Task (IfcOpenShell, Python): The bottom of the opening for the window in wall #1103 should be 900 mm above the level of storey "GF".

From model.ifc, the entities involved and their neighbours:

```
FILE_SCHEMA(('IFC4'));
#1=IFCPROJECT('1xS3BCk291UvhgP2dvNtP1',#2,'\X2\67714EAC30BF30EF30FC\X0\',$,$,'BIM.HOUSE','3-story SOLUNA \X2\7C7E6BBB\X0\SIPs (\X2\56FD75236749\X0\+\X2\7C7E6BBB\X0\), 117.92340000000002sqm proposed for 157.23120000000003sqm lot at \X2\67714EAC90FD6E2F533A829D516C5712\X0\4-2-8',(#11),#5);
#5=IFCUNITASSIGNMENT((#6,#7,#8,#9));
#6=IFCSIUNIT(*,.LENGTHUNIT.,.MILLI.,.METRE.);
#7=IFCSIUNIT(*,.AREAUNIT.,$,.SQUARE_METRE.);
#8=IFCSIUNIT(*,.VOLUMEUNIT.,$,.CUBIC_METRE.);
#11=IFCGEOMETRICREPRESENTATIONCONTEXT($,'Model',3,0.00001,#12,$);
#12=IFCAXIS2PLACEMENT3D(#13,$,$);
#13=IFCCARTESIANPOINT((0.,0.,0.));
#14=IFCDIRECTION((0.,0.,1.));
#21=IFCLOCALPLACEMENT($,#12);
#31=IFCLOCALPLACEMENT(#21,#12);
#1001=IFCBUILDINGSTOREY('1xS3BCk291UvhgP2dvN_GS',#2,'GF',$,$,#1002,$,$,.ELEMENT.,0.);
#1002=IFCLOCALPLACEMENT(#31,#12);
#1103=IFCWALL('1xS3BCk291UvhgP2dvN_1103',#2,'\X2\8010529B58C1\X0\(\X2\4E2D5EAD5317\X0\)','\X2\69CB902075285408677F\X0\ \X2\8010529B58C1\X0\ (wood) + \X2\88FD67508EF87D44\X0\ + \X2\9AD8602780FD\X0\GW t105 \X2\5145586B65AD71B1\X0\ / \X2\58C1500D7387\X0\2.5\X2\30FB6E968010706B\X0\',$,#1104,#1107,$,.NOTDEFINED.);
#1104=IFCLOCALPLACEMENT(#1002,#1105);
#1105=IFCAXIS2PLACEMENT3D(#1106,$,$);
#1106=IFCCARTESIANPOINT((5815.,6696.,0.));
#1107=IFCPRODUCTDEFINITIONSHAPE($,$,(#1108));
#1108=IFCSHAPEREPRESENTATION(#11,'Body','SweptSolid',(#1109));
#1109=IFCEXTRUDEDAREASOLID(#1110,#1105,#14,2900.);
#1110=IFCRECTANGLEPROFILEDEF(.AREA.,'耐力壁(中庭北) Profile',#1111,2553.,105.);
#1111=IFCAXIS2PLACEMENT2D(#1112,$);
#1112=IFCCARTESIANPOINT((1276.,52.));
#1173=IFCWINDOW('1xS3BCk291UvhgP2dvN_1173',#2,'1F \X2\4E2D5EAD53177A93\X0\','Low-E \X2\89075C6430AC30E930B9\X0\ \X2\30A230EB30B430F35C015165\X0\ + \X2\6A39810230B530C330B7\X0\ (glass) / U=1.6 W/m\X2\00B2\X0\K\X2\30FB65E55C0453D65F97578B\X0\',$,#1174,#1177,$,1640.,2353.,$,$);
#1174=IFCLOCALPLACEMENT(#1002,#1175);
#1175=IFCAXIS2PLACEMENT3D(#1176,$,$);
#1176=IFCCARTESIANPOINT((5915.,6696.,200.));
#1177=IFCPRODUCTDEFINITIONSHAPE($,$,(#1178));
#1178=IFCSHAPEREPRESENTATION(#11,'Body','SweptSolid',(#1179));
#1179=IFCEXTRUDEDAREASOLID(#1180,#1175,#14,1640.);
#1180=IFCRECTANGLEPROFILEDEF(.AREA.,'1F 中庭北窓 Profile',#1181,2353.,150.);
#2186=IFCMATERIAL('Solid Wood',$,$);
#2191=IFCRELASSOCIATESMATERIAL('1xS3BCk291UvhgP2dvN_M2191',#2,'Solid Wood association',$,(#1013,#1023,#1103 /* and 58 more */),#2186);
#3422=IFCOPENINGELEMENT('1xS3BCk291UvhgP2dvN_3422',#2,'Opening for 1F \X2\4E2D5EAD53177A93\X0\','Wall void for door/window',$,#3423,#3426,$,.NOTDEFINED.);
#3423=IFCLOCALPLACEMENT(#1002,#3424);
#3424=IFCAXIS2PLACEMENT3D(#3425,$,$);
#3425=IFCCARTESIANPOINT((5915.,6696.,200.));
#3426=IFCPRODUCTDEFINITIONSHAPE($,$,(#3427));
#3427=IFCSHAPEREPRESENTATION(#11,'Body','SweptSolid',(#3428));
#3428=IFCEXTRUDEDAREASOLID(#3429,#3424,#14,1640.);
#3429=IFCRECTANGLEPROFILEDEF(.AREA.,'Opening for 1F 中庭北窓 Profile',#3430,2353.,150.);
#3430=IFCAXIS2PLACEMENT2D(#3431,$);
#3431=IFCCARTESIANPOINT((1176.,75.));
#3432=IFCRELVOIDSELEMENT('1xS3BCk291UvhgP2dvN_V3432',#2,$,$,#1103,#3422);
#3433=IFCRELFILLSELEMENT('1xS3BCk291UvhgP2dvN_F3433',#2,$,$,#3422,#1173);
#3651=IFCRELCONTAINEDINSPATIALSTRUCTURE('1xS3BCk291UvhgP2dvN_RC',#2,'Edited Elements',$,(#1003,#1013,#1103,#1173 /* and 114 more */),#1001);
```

```python
import numpy as np
import ifcopenshell
import ifcopenshell.api.geometry
import ifcopenshell.geom
import ifcopenshell.util.element
import ifcopenshell.util.placement
import ifcopenshell.util.shape
import ifcopenshell.util.unit

model = ifcopenshell.open("model.ifc")
unit_scale = ifcopenshell.util.unit.calculate_unit_scale(model)

window = model.by_guid("1xS3BCk291UvhgP2dvN_1173")
opening = window.FillsVoids[0].RelatingOpeningElement
storey = ifcopenshell.util.element.get_container(window, ifc_class="IfcBuildingStorey")
level = ifcopenshell.util.placement.get_local_placement(storey.ObjectPlacement)[2, 3]

# The opening's origin need not be at the sill, so measure its lowest point.
shape = ifcopenshell.geom.create_shape(ifcopenshell.geom.settings(), opening)
bottom = ifcopenshell.util.shape.get_shape_bottom_elevation(shape, shape.geometry) / unit_scale
dz = level + 900.0 - bottom

shift = np.array([0.0, 0.0, dz])
# The window is not placed relative to its opening, so move both.
for product in (opening, window):
    matrix = ifcopenshell.util.placement.get_local_placement(product.ObjectPlacement)
    matrix[:3, 3] += shift
    ifcopenshell.api.geometry.edit_object_placement(model, product=product, matrix=matrix, is_si=False)

print(f"moved by {dz * unit_scale:+.3f} m")

model.write("model-out.ifc")
```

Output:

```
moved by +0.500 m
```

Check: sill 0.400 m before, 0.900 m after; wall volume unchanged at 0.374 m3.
